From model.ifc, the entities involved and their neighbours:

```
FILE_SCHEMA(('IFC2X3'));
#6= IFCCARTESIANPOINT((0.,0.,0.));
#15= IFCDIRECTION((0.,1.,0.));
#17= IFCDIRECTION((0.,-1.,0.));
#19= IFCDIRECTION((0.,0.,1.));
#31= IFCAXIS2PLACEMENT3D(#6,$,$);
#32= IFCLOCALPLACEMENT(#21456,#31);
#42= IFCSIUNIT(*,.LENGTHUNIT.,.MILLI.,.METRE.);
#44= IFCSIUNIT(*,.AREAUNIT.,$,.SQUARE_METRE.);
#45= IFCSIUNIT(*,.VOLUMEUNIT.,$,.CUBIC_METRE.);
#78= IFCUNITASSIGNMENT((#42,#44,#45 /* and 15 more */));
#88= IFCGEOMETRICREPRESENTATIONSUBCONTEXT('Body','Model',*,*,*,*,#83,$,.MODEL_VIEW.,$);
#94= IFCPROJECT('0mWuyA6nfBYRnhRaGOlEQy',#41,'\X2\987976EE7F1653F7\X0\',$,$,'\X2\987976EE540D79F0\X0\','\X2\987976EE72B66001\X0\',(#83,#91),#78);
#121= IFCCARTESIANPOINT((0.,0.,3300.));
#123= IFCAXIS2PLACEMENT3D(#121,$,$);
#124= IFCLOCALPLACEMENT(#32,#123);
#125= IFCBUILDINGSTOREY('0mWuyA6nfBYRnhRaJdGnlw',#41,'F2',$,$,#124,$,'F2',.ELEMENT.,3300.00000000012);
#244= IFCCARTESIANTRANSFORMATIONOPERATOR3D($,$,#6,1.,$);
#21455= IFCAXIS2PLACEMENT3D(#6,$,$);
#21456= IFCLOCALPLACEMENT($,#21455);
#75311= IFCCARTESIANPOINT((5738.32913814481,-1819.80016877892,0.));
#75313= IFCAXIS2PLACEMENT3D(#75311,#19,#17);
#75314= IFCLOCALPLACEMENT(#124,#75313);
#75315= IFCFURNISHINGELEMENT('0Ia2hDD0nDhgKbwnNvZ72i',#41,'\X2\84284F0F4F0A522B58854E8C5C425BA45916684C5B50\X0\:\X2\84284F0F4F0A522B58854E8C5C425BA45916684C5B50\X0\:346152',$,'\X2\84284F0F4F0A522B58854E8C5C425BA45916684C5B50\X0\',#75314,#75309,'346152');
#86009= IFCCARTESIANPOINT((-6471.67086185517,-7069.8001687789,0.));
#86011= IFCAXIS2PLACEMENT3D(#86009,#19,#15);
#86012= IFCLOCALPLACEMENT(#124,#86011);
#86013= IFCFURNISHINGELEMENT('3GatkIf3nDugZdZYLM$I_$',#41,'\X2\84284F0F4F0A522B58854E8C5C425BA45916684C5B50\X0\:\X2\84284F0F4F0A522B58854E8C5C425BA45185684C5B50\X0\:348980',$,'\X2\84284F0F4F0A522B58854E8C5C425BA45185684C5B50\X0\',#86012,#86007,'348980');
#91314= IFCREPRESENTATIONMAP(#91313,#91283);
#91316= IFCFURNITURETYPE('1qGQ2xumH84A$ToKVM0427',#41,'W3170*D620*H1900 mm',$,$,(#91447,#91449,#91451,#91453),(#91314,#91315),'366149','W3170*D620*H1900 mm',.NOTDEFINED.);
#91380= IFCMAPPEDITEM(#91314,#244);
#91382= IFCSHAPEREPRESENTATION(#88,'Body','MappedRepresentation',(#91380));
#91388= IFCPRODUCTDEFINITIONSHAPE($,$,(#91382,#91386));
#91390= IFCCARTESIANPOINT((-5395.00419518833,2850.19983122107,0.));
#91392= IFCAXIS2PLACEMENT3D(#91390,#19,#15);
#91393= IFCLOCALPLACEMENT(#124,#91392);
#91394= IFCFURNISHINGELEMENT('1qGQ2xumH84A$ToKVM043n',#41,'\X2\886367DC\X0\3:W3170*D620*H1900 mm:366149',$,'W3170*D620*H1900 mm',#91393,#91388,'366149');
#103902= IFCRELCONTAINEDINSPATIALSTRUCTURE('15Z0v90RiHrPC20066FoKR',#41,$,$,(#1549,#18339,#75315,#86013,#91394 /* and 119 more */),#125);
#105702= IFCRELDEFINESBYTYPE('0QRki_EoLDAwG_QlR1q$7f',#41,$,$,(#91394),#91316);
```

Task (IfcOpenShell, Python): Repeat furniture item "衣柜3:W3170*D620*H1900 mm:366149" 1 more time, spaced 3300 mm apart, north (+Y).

```python
import numpy as np
import ifcopenshell
import ifcopenshell.api.geometry
import ifcopenshell.api.root
import ifcopenshell.util.element
import ifcopenshell.util.placement
import ifcopenshell.util.unit

model = ifcopenshell.open("model.ifc")
unit_scale = ifcopenshell.util.unit.calculate_unit_scale(model)


def reuse_history(source, copy):
    """copy_class also copies each property set's owner history, people and application; keep the originals."""
    for rel in copy.IsDefinedBy:
        if rel.is_a("IfcRelDefinesByProperties") and (history := rel.RelatingPropertyDefinition.OwnerHistory):
            rel.RelatingPropertyDefinition.OwnerHistory = source.OwnerHistory
            ifcopenshell.util.element.remove_deep2(model, history)


source = model.by_guid("1qGQ2xumH84A$ToKVM043n")
base = ifcopenshell.util.placement.get_local_placement(source.ObjectPlacement)
step = np.array([0.0, 1.0, 0.0]) * 3.3 / unit_scale

for i in range(1, 2):
    copy = ifcopenshell.api.root.copy_class(model, product=source)
    copy.Representation = ifcopenshell.util.element.copy_deep(
        model, source.Representation, exclude=["IfcGeometricRepresentationContext", "IfcRepresentationMap"]
    )
    copy.Name = "衣柜3:W3170*D620*H1900 mm"
    copy.Tag = None
    reuse_history(source, copy)
    matrix = base.copy()
    matrix[:3, 3] += i * step
    print("added at", matrix[:3, 3].round(3) + 0.0)
    ifcopenshell.api.geometry.edit_object_placement(model, product=copy, matrix=matrix, is_si=False)

model.write("model_v2.ifc")
```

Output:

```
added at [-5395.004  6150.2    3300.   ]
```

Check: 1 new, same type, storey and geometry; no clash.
